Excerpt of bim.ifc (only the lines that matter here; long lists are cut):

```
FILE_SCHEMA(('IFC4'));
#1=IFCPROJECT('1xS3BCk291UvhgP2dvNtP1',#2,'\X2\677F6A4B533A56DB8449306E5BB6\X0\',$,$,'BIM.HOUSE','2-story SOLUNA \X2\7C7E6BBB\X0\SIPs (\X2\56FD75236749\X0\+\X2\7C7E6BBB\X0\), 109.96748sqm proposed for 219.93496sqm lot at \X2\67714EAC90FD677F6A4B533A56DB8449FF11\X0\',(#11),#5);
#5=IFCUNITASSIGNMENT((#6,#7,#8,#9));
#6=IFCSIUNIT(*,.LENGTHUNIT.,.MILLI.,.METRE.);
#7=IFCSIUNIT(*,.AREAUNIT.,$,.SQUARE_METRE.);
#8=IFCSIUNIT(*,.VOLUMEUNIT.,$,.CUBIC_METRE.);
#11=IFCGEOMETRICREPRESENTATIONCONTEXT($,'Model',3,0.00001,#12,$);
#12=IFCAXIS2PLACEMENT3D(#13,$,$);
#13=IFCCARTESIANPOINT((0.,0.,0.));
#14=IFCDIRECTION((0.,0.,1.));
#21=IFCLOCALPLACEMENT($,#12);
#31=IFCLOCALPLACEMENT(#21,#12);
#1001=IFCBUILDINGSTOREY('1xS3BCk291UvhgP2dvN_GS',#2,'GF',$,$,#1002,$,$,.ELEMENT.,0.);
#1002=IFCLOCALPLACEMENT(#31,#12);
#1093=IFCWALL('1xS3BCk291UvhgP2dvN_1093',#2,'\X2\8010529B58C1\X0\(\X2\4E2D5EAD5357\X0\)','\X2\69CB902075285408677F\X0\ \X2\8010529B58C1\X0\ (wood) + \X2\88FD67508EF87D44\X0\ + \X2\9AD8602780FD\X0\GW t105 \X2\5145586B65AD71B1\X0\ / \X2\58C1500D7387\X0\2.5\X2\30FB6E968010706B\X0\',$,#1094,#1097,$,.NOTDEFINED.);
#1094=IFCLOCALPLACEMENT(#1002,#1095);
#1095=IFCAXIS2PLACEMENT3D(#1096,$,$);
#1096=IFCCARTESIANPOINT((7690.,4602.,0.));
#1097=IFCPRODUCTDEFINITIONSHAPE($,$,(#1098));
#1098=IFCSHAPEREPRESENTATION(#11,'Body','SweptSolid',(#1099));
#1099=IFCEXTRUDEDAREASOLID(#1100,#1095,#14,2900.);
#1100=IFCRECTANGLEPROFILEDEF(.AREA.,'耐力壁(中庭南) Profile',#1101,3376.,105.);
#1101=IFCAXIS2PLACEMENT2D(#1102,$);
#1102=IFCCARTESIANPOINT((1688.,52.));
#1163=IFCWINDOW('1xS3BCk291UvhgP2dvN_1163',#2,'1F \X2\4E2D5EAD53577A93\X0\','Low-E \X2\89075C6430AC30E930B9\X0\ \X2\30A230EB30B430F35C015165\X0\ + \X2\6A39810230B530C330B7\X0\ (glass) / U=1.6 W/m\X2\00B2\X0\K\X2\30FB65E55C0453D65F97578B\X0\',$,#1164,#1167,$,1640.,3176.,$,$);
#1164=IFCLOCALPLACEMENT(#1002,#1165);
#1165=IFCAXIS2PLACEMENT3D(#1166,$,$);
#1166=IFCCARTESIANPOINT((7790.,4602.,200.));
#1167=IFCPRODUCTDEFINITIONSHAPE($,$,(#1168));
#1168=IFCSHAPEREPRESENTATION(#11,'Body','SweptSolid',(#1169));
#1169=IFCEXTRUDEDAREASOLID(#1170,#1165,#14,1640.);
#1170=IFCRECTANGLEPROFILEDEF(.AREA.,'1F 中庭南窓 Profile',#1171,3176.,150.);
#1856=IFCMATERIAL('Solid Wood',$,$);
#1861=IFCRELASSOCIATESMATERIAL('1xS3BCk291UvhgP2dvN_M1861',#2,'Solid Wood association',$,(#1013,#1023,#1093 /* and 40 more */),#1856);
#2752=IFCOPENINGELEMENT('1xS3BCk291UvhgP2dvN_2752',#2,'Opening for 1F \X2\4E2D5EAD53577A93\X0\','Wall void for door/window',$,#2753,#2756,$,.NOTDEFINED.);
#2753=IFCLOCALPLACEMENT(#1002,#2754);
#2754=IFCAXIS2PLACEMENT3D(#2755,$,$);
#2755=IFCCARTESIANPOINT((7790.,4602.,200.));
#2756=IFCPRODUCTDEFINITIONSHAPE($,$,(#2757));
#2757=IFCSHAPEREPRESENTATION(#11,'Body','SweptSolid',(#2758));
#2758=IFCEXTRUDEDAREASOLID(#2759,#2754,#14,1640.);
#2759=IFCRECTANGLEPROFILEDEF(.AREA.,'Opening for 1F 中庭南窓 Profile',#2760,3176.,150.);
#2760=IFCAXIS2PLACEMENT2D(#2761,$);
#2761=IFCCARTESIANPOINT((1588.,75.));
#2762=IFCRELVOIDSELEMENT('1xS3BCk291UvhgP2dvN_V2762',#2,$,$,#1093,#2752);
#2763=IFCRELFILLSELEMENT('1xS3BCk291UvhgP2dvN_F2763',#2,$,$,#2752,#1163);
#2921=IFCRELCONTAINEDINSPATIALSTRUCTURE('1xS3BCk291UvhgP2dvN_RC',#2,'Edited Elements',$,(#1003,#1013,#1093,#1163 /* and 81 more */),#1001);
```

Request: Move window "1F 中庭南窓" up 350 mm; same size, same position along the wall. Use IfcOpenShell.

```python
import numpy as np
import ifcopenshell
import ifcopenshell.api.geometry
import ifcopenshell.util.placement
import ifcopenshell.util.unit

model = ifcopenshell.open("bim.ifc")
unit_scale = ifcopenshell.util.unit.calculate_unit_scale(model)

window = model.by_id(1163)
opening = window.FillsVoids[0].RelatingOpeningElement
dz = 350.0

shift = np.array([0.0, 0.0, dz])
# The window is not placed relative to its opening, so move both.
for product in (opening, window):
    matrix = ifcopenshell.util.placement.get_local_placement(product.ObjectPlacement)
    matrix[:3, 3] += shift
    ifcopenshell.api.geometry.edit_object_placement(model, product=product, matrix=matrix, is_si=False)

print(f"moved by {dz * unit_scale:+.3f} m")

model.write("bim_v2.ifc")
```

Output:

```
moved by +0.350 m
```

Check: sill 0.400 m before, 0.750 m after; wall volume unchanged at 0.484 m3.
